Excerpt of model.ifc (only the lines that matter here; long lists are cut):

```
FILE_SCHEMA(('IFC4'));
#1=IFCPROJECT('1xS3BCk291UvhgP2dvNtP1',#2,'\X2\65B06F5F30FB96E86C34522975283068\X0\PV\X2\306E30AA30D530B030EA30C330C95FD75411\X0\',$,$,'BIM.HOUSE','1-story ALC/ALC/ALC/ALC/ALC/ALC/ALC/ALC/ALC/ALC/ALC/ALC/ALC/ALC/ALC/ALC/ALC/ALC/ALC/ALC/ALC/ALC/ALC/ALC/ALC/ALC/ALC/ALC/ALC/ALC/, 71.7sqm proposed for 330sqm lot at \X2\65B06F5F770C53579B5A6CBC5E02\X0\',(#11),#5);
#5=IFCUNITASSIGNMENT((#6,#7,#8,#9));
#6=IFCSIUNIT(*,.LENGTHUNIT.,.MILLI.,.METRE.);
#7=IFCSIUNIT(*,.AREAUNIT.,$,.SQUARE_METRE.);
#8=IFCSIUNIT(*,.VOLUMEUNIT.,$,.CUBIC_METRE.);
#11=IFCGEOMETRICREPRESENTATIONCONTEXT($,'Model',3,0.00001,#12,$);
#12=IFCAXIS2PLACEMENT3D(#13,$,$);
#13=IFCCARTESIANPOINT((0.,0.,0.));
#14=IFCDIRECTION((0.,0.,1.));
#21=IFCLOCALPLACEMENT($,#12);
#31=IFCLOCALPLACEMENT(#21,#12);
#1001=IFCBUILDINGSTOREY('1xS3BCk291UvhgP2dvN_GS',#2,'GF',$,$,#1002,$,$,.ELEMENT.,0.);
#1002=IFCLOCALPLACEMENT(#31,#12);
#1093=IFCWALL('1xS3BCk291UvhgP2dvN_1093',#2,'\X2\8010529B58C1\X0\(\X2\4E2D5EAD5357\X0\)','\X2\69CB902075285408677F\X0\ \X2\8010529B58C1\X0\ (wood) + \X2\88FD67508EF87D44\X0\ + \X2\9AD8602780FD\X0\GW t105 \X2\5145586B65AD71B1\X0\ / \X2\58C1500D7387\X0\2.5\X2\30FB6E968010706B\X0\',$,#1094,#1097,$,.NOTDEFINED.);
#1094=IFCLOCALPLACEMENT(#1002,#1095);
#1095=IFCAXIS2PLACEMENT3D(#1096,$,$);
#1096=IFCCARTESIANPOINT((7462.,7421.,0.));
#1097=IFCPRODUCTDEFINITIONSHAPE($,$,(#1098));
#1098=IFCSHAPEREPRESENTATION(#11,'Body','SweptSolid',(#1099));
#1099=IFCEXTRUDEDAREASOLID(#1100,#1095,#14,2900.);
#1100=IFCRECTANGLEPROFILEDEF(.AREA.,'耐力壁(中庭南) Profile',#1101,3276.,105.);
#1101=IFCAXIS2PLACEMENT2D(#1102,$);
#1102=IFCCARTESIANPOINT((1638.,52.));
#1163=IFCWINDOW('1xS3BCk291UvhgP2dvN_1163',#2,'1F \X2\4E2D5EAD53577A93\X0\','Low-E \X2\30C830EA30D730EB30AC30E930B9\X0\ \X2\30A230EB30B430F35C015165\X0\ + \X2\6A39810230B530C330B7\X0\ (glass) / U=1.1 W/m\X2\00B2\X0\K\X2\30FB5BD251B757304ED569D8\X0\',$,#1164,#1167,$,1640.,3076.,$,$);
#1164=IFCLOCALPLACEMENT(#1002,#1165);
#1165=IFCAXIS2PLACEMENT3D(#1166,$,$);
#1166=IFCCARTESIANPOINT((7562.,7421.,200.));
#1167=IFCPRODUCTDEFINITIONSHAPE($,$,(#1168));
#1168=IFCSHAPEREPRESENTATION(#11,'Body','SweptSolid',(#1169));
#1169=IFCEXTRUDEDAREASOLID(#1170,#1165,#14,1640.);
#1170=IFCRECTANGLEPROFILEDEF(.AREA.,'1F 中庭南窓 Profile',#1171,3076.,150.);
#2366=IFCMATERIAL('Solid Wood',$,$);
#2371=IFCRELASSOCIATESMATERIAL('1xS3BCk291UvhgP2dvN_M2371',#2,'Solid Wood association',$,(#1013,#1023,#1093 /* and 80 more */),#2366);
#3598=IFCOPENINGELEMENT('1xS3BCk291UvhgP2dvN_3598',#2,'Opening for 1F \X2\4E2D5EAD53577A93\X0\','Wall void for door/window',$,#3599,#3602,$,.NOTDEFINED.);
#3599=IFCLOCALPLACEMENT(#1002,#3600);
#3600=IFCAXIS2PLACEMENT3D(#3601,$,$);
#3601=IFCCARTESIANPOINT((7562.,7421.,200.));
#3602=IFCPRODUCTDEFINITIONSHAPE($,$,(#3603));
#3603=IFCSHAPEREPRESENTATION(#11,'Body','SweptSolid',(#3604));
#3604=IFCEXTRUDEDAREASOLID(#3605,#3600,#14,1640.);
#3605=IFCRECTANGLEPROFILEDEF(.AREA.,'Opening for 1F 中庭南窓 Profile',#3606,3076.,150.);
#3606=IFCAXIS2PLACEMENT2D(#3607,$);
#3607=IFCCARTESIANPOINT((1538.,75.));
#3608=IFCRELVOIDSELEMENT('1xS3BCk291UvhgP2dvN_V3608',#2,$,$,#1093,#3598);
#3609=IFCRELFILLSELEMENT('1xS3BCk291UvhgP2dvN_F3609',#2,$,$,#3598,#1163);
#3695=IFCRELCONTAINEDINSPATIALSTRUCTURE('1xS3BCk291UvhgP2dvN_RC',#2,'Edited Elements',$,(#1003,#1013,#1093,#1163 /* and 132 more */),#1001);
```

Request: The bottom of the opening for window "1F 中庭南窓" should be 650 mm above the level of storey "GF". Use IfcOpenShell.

```python
import numpy as np
import ifcopenshell
import ifcopenshell.api.geometry
import ifcopenshell.geom
import ifcopenshell.util.element
import ifcopenshell.util.placement
import ifcopenshell.util.shape
import ifcopenshell.util.unit

model = ifcopenshell.open("model.ifc")
unit_scale = ifcopenshell.util.unit.calculate_unit_scale(model)

window = model.by_guid("1xS3BCk291UvhgP2dvN_1163")
opening = window.FillsVoids[0].RelatingOpeningElement
storey = ifcopenshell.util.element.get_container(window, ifc_class="IfcBuildingStorey")
level = ifcopenshell.util.placement.get_local_placement(storey.ObjectPlacement)[2, 3]

# The opening's origin need not be at the sill, so measure its lowest point.
shape = ifcopenshell.geom.create_shape(ifcopenshell.geom.settings(), opening)
bottom = ifcopenshell.util.shape.get_shape_bottom_elevation(shape, shape.geometry) / unit_scale
dz = level + 0.65 / unit_scale - bottom

shift = np.array([0.0, 0.0, dz])
# The window is not placed relative to its opening, so move both.
for product in (opening, window):
    matrix = ifcopenshell.util.placement.get_local_placement(product.ObjectPlacement)
    matrix[:3, 3] += shift
    ifcopenshell.api.geometry.edit_object_placement(model, product=product, matrix=matrix, is_si=False)

print(f"moved by {dz * unit_scale:+.3f} m")

model.write("model_rev.ifc")
```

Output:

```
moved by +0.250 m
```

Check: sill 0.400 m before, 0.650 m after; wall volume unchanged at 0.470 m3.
